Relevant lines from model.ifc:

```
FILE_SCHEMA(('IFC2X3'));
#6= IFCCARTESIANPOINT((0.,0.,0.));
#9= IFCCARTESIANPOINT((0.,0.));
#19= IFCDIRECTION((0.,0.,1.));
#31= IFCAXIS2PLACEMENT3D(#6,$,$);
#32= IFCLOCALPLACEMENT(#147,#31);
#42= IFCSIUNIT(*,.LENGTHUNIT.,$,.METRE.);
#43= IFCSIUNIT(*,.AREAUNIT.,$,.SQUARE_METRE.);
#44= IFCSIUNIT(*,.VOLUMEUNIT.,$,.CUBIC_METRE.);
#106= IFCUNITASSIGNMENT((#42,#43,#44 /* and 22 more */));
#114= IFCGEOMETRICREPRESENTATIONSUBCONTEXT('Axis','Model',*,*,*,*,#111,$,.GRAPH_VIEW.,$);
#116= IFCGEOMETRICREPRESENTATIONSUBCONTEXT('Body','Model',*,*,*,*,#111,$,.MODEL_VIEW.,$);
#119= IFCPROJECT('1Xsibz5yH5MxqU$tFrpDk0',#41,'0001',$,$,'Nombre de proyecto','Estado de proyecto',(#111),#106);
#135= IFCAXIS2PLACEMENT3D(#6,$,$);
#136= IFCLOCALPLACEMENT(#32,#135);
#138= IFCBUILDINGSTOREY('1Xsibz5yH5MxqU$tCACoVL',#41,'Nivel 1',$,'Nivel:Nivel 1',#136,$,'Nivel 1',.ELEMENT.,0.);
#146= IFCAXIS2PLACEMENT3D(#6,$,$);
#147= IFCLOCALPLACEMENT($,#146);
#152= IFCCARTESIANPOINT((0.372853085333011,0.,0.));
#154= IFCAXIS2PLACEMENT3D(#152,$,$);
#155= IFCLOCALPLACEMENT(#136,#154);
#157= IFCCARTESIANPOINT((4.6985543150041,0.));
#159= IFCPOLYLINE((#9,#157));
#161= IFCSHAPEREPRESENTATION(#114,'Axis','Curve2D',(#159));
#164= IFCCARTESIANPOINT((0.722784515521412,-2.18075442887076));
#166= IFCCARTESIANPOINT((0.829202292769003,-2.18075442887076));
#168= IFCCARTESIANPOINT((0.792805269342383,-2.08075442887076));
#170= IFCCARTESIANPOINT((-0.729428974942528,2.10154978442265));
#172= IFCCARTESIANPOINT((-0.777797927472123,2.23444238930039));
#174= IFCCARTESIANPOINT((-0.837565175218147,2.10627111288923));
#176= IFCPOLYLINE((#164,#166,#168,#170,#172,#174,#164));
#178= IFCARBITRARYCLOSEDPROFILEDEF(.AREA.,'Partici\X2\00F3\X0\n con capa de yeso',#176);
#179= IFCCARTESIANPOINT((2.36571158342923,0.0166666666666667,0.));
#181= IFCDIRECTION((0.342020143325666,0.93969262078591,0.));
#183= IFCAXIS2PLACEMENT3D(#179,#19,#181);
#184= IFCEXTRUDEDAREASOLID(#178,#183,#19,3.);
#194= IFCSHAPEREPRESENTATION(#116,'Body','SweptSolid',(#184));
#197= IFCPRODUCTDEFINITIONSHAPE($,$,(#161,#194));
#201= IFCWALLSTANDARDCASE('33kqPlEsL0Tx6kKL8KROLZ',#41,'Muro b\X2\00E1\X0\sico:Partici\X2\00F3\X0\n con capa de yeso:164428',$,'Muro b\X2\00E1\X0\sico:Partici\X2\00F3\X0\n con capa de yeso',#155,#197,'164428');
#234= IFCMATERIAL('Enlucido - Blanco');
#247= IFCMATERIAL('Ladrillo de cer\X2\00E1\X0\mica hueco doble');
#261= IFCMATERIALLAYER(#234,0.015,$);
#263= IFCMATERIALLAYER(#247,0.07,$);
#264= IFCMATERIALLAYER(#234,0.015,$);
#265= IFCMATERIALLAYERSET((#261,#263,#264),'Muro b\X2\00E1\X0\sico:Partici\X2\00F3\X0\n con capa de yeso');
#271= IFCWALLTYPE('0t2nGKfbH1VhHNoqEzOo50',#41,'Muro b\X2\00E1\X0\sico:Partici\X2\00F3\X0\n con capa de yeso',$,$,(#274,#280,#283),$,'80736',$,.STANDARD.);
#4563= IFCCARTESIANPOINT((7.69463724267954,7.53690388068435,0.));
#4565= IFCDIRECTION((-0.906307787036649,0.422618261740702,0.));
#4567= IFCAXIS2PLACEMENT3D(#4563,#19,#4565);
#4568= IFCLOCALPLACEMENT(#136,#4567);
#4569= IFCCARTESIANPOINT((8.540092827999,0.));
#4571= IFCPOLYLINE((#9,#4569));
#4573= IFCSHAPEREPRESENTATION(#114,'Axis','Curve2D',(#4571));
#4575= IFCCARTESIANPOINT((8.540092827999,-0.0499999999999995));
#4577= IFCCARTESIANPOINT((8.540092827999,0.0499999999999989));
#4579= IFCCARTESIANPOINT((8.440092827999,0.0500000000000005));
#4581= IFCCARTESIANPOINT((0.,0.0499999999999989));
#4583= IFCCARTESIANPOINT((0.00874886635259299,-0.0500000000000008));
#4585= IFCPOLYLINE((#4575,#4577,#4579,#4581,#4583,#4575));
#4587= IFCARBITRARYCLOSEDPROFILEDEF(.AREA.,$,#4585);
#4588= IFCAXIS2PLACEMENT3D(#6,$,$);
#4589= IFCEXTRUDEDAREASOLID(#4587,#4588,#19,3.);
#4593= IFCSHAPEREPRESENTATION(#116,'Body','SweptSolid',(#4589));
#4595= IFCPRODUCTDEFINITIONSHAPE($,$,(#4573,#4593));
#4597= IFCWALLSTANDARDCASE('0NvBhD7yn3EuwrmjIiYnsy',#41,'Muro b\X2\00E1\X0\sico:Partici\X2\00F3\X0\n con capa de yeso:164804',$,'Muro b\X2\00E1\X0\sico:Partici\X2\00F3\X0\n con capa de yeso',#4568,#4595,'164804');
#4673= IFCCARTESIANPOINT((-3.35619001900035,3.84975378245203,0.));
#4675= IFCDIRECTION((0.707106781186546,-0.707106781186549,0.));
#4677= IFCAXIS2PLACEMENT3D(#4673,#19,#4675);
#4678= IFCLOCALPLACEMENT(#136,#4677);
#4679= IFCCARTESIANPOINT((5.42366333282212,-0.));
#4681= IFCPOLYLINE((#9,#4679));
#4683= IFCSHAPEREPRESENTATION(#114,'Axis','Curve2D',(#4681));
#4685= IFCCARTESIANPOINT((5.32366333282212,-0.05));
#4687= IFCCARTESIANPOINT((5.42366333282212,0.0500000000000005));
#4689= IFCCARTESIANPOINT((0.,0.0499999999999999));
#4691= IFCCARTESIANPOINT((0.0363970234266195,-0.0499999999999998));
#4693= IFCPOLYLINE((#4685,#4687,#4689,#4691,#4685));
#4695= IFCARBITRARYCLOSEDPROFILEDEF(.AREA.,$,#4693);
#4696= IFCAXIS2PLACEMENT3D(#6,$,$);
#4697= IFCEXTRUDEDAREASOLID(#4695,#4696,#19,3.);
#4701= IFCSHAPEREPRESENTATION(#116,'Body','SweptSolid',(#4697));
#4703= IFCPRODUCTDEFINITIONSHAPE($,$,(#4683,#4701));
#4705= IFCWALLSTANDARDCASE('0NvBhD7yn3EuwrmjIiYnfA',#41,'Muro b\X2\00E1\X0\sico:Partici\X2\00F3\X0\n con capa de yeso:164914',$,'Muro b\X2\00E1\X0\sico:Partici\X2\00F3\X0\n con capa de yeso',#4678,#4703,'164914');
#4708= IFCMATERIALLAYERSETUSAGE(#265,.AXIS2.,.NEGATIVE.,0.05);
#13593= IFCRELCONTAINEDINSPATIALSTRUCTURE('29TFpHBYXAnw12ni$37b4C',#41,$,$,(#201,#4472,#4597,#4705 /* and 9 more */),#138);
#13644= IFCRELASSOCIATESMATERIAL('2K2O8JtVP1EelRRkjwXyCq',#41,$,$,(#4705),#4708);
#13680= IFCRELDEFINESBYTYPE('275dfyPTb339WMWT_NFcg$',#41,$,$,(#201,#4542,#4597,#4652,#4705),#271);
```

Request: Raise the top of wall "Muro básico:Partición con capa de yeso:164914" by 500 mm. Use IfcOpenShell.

```python
import ifcopenshell
import ifcopenshell.geom
import ifcopenshell.util.representation
import ifcopenshell.util.shape
import ifcopenshell.util.unit

model = ifcopenshell.open("model.ifc")
unit_scale = ifcopenshell.util.unit.calculate_unit_scale(model)
settings = ifcopenshell.geom.settings()


def volume(element):
    """Net volume in cubic metres, openings subtracted."""
    shape = ifcopenshell.geom.create_shape(settings, element)
    return ifcopenshell.util.shape.get_volume(shape.geometry)


wall = model.by_guid("0NvBhD7yn3EuwrmjIiYnfA")
before = volume(wall)

body = ifcopenshell.util.representation.get_representation(wall, "Model", "Body")
solid = body.Items[0]
old_height = solid.Depth
solid.Depth += 0.5 / unit_scale
after = volume(wall)

print(f"height {old_height:g} -> {solid.Depth:g}, volume {before:.3f} -> {after:.3f} m3")

model.write("model-out.ifc")
```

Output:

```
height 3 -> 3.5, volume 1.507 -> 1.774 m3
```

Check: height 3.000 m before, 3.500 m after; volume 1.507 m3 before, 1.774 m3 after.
